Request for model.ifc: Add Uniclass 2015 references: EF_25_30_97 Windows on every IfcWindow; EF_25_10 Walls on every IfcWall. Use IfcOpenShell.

First a look at what the model holds.

```python
import ifcopenshell

model = ifcopenshell.open("model.ifc")
print(model.schema)
print("classifications:", [c.Name for c in model.by_type("IfcClassification")])
for ifc_class in ("IfcDoor", "IfcRoof", "IfcStair", "IfcWall", "IfcWindow"):
    print(ifc_class, len(model.by_type(ifc_class)))
```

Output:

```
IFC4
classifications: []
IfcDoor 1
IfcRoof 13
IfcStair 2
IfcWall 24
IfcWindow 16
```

```python
import ifcopenshell
import ifcopenshell.api.classification

model = ifcopenshell.open("model.ifc")

system = ifcopenshell.api.classification.add_classification(model, classification="Uniclass 2015")

codes = {
    "IfcWindow": ("EF_25_30_97", "Windows"),
    "IfcWall": ("EF_25_10", "Walls"),
}
for ifc_class, (code, name) in codes.items():
    products = model.by_type(ifc_class)
    ifcopenshell.api.classification.add_reference(
        model, products=products, classification=system, identification=code, name=name
    )
    print(code, len(products))

model.write("model_edited.ifc")
```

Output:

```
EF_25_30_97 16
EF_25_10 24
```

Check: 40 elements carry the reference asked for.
